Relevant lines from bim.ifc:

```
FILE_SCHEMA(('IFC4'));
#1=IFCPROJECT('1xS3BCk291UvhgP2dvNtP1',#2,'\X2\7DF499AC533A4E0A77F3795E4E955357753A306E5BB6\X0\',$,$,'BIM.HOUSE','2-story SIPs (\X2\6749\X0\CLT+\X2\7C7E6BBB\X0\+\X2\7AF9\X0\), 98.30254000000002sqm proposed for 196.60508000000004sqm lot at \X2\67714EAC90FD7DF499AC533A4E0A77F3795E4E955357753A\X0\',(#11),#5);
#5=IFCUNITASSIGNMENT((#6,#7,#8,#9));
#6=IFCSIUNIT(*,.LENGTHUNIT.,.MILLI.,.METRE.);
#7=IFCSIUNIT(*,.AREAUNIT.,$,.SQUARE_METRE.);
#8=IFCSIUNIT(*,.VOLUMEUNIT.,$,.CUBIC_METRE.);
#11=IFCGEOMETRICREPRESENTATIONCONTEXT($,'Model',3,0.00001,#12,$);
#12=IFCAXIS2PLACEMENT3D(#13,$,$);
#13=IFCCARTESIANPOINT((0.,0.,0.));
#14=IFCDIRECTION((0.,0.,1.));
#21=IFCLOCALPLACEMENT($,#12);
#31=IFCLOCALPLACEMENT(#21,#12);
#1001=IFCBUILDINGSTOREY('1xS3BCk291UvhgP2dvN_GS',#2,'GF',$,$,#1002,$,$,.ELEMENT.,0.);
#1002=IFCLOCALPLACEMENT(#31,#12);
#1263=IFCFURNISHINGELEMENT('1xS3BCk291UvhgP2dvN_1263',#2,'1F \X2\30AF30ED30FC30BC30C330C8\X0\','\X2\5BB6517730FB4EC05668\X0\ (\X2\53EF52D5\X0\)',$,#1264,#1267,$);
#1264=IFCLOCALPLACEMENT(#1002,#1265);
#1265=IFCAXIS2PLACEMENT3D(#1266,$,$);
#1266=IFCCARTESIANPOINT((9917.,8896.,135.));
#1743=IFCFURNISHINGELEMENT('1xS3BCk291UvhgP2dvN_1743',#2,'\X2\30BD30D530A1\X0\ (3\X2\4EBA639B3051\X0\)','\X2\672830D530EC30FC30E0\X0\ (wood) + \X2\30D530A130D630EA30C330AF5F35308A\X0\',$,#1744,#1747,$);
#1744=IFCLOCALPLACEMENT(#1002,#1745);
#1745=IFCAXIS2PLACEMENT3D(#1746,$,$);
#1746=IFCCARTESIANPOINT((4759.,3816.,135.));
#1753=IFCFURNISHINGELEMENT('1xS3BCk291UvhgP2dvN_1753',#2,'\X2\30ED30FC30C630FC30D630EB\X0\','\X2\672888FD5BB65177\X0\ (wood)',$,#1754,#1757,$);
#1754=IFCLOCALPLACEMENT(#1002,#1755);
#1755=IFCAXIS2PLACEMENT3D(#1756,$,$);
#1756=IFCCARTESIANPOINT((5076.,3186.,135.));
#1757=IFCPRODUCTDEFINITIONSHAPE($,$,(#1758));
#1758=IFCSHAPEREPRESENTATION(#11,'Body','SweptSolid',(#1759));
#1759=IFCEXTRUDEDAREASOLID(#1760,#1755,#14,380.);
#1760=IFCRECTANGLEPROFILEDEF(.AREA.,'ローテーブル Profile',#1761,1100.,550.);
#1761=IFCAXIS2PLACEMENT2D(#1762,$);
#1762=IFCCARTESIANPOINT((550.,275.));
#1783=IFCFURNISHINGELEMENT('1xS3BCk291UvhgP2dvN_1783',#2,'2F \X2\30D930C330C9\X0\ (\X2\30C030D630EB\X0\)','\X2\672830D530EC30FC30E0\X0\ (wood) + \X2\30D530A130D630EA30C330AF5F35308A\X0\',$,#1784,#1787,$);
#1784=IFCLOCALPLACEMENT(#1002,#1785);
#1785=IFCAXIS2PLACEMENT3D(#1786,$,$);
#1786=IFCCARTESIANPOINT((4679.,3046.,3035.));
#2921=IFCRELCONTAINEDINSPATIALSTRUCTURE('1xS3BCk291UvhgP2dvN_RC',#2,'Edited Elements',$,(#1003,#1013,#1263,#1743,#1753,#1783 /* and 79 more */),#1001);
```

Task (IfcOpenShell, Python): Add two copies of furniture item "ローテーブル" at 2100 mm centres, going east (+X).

```python
import numpy as np
import ifcopenshell
import ifcopenshell.api.geometry
import ifcopenshell.api.root
import ifcopenshell.util.element
import ifcopenshell.util.placement

model = ifcopenshell.open("bim.ifc")


def reuse_history(source, copy):
    """copy_class also copies each property set's owner history, people and application; keep the originals."""
    for rel in copy.IsDefinedBy:
        if rel.is_a("IfcRelDefinesByProperties") and (history := rel.RelatingPropertyDefinition.OwnerHistory):
            rel.RelatingPropertyDefinition.OwnerHistory = source.OwnerHistory
            ifcopenshell.util.element.remove_deep2(model, history)


source = model.by_guid("1xS3BCk291UvhgP2dvN_1753")
base = ifcopenshell.util.placement.get_local_placement(source.ObjectPlacement)
step = np.array([1.0, 0.0, 0.0]) * 2100.0

for i in range(1, 3):
    copy = ifcopenshell.api.root.copy_class(model, product=source)
    copy.Representation = ifcopenshell.util.element.copy_deep(
        model, source.Representation, exclude=["IfcGeometricRepresentationContext", "IfcRepresentationMap"]
    )
    reuse_history(source, copy)
    matrix = base.copy()
    matrix[:3, 3] += i * step
    print("added at", matrix[:3, 3].round(3) + 0.0)
    ifcopenshell.api.geometry.edit_object_placement(model, product=copy, matrix=matrix, is_si=False)

model.write("bim_updated.ifc")
```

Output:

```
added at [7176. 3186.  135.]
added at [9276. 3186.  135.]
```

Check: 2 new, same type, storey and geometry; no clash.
